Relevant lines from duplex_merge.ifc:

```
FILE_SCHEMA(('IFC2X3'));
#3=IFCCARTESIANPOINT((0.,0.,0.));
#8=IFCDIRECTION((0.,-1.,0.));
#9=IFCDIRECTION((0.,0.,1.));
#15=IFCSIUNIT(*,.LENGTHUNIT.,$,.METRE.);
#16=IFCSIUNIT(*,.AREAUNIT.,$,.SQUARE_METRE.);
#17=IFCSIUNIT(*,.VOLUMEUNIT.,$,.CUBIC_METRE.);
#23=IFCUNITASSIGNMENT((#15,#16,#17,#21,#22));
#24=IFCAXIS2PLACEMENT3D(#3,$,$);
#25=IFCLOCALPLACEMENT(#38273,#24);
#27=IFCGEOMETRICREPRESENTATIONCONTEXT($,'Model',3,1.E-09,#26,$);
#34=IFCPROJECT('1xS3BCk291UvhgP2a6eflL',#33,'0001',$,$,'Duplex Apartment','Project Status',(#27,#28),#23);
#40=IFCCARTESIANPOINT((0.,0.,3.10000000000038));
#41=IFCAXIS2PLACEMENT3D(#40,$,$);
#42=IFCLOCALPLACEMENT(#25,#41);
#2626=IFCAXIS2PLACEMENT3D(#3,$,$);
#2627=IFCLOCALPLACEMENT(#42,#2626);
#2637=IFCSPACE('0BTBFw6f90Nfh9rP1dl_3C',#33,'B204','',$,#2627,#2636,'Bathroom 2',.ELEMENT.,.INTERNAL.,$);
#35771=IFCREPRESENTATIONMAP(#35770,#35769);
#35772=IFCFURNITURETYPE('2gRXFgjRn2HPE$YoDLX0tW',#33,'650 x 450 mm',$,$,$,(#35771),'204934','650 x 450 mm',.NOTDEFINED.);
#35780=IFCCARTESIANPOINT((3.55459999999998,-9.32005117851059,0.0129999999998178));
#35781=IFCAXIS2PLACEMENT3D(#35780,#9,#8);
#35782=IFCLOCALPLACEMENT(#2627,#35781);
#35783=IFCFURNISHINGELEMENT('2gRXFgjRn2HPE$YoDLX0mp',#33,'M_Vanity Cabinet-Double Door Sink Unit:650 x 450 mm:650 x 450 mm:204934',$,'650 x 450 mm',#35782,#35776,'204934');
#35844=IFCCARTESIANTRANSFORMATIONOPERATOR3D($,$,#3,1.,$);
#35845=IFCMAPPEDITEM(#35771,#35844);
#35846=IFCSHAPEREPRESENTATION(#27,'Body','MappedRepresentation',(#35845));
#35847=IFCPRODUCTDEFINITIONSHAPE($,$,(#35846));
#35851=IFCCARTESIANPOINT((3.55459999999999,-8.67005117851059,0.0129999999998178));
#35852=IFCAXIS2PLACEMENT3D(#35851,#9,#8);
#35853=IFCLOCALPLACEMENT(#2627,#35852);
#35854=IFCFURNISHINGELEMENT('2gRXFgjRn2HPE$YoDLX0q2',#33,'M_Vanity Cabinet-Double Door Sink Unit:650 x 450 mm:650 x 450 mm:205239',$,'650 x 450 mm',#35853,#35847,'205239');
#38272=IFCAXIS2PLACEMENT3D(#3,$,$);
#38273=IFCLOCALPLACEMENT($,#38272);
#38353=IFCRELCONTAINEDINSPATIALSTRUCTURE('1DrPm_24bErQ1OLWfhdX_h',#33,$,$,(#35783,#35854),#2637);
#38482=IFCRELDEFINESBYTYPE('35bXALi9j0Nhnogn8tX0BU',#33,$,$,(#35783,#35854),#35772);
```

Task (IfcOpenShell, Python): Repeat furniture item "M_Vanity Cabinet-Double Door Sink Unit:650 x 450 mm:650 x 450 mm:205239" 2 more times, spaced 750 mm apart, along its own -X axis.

```python
import ifcopenshell
import ifcopenshell.api.geometry
import ifcopenshell.api.root
import ifcopenshell.util.element
import ifcopenshell.util.placement

model = ifcopenshell.open("duplex_merge.ifc")


def reuse_history(source, copy):
    """copy_class also copies each property set's owner history, people and application; keep the originals."""
    for rel in copy.IsDefinedBy:
        if rel.is_a("IfcRelDefinesByProperties") and (history := rel.RelatingPropertyDefinition.OwnerHistory):
            rel.RelatingPropertyDefinition.OwnerHistory = source.OwnerHistory
            ifcopenshell.util.element.remove_deep2(model, history)


source = model.by_guid("2gRXFgjRn2HPE$YoDLX0q2")
base = ifcopenshell.util.placement.get_local_placement(source.ObjectPlacement)
step = -base[:3, 0] * 0.75

for i in range(1, 3):
    copy = ifcopenshell.api.root.copy_class(model, product=source)
    copy.Representation = ifcopenshell.util.element.copy_deep(
        model, source.Representation, exclude=["IfcGeometricRepresentationContext", "IfcRepresentationMap"]
    )
    copy.Name = "M_Vanity Cabinet-Double Door Sink Unit:650 x 450 mm:650 x 450 mm"
    copy.Tag = None
    reuse_history(source, copy)
    matrix = base.copy()
    matrix[:3, 3] += i * step
    print("added at", matrix[:3, 3].round(3) + 0.0)
    ifcopenshell.api.geometry.edit_object_placement(model, product=copy, matrix=matrix, is_si=False)

model.write("duplex_merge_v2.ifc")
```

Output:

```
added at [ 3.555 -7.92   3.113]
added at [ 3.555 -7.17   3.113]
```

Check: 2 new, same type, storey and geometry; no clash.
